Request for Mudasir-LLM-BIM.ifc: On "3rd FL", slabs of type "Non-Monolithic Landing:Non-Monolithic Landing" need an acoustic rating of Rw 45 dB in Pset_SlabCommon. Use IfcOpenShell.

First a look at what the model holds.

```python
import ifcopenshell
import ifcopenshell.util.element

model = ifcopenshell.open("Mudasir-LLM-BIM.ifc")
print(model.schema)
storey = next(s for s in model.by_type("IfcBuildingStorey") if s.Name == "3rd FL")
slabs = [e for e in ifcopenshell.util.element.get_decomposition(storey) if e.is_a("IfcSlab")]
seen = {}
for e in slabs:
    element_type = ifcopenshell.util.element.get_type(e)
    key = (element_type.Name if element_type != e and element_type else None, ifcopenshell.util.element.get_pset(e, "Pset_SlabCommon", "AcousticRating"))
    seen[key] = seen.get(key, 0) + 1
for (name, value), count in sorted(seen.items(), key=str):
    print(count, "x", name, "|", value)
```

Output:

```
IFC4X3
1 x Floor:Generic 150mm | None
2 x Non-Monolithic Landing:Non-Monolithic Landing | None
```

```python
import ifcopenshell
import ifcopenshell.api.pset
import ifcopenshell.util.element

model = ifcopenshell.open("Mudasir-LLM-BIM.ifc")

storey = next(s for s in model.by_type("IfcBuildingStorey") if s.Name == "3rd FL")
slabs = [e for e in ifcopenshell.util.element.get_decomposition(storey) if e.is_a("IfcSlab")]

count = 0
for e in slabs:
    element_type = ifcopenshell.util.element.get_type(e)
    if element_type in (None, e) or element_type.Name != "Non-Monolithic Landing:Non-Monolithic Landing":
        continue
    # add_pset returns the element's existing set when there is one.
    pset = ifcopenshell.api.pset.add_pset(model, product=e, name="Pset_SlabCommon")
    ifcopenshell.api.pset.edit_pset(model, pset=pset, properties={"AcousticRating": "Rw 45 dB"})
    count += 1

print(count, "slabs updated")

model.write("Mudasir-LLM-BIM_edited.ifc")
```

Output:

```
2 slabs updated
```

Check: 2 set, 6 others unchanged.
